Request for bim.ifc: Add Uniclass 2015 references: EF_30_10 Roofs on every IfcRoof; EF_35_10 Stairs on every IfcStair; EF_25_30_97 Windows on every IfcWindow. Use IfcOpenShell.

First a look at what the model holds.

```python
import ifcopenshell

model = ifcopenshell.open("bim.ifc")
print(model.schema)
print("classifications:", [c.Name for c in model.by_type("IfcClassification")])
for ifc_class in ("IfcDoor", "IfcRoof", "IfcStair", "IfcWall", "IfcWindow"):
    print(ifc_class, len(model.by_type(ifc_class)))
```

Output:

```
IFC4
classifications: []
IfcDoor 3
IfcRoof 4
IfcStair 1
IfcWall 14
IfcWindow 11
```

```python
import ifcopenshell
import ifcopenshell.api.classification

model = ifcopenshell.open("bim.ifc")

system = ifcopenshell.api.classification.add_classification(model, classification="Uniclass 2015")

codes = {
    "IfcRoof": ("EF_30_10", "Roofs"),
    "IfcStair": ("EF_35_10", "Stairs"),
    "IfcWindow": ("EF_25_30_97", "Windows"),
}
for ifc_class, (code, name) in codes.items():
    products = model.by_type(ifc_class)
    ifcopenshell.api.classification.add_reference(
        model, products=products, classification=system, identification=code, name=name
    )
    print(code, len(products))

model.write("bim_edited.ifc")
```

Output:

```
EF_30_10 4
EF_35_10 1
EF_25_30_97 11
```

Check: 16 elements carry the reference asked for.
